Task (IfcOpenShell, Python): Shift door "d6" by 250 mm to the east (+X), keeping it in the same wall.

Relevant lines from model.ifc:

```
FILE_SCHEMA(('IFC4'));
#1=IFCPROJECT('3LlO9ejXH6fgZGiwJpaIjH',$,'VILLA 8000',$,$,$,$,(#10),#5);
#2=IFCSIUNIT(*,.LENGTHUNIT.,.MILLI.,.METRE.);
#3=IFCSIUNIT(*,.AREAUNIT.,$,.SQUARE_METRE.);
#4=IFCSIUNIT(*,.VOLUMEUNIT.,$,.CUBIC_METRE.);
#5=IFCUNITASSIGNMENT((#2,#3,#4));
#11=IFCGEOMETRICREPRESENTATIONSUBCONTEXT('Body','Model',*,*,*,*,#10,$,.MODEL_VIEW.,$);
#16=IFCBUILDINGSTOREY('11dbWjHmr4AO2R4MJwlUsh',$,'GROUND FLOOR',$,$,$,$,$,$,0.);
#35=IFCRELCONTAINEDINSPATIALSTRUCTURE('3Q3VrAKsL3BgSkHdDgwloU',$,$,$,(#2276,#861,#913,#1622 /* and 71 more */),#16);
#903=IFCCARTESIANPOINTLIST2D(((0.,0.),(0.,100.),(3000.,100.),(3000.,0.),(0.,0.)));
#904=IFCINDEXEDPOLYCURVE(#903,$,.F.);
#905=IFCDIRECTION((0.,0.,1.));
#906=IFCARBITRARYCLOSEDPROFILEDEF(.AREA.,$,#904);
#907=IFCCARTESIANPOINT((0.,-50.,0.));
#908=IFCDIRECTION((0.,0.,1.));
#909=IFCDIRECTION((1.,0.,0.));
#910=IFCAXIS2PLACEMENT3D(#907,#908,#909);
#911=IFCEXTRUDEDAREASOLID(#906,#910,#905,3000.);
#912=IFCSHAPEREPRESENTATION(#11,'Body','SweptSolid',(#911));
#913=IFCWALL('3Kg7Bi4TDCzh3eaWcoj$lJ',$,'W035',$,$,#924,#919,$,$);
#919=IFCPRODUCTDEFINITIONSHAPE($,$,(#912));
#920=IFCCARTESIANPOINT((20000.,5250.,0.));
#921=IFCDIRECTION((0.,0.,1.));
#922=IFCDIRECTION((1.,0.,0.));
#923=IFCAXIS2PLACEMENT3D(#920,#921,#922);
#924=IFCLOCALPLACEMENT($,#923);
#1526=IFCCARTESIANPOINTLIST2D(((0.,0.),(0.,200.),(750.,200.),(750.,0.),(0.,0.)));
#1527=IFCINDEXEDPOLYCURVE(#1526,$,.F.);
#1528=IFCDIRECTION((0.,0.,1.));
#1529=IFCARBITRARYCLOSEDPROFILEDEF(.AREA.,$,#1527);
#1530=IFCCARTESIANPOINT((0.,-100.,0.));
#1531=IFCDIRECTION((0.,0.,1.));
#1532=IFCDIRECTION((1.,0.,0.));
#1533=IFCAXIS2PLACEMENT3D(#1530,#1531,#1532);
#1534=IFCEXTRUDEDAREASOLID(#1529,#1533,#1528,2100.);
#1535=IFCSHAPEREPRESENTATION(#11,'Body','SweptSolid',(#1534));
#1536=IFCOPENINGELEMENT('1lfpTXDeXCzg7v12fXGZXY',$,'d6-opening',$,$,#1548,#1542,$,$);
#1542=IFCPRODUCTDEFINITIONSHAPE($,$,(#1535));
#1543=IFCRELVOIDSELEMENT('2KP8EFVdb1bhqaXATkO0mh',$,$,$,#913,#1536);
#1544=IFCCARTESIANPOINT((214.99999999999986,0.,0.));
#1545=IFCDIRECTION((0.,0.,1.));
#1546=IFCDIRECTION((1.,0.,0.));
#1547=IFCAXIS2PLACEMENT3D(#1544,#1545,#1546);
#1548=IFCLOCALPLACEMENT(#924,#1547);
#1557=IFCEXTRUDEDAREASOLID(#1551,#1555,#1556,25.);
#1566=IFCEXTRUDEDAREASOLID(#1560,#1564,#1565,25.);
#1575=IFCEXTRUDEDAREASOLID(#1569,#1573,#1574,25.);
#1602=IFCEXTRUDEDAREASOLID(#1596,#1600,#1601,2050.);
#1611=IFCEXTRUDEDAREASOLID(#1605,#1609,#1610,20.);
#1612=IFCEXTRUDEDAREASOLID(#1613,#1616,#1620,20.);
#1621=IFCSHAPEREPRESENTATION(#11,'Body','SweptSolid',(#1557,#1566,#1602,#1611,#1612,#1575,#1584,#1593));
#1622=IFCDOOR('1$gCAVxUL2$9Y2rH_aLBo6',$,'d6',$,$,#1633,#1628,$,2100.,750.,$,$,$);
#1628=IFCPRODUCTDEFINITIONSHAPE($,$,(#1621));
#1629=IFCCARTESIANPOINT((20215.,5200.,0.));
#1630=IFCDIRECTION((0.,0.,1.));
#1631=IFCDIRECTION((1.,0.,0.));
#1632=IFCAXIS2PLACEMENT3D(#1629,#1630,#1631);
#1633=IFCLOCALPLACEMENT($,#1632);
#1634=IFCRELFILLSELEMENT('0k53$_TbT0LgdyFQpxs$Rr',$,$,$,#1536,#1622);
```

```python
import ifcopenshell
import ifcopenshell.api.geometry
import ifcopenshell.util.placement

model = ifcopenshell.open("model.ifc")

door = model.by_guid("1$gCAVxUL2$9Y2rH_aLBo6")
opening = door.FillsVoids[0].RelatingOpeningElement
wall = opening.VoidsElements[0].RelatingBuildingElement

wall_matrix = ifcopenshell.util.placement.get_local_placement(wall.ObjectPlacement)
shift = wall_matrix[:3, 0] * 250.0
before = ifcopenshell.util.placement.get_local_placement(door.ObjectPlacement)[:3, 3].copy()

# The door is not placed relative to its opening, so move both.
for product in (opening, door):
    matrix = ifcopenshell.util.placement.get_local_placement(product.ObjectPlacement)
    matrix[:3, 3] += shift
    ifcopenshell.api.geometry.edit_object_placement(model, product=product, matrix=matrix, is_si=False)

after = ifcopenshell.util.placement.get_local_placement(door.ObjectPlacement)[:3, 3]
print("door moved by", (after - before).round(3) + 0.0)

model.write("model_rev.ifc")
```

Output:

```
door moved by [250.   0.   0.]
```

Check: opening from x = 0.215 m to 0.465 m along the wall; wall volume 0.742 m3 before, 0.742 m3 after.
